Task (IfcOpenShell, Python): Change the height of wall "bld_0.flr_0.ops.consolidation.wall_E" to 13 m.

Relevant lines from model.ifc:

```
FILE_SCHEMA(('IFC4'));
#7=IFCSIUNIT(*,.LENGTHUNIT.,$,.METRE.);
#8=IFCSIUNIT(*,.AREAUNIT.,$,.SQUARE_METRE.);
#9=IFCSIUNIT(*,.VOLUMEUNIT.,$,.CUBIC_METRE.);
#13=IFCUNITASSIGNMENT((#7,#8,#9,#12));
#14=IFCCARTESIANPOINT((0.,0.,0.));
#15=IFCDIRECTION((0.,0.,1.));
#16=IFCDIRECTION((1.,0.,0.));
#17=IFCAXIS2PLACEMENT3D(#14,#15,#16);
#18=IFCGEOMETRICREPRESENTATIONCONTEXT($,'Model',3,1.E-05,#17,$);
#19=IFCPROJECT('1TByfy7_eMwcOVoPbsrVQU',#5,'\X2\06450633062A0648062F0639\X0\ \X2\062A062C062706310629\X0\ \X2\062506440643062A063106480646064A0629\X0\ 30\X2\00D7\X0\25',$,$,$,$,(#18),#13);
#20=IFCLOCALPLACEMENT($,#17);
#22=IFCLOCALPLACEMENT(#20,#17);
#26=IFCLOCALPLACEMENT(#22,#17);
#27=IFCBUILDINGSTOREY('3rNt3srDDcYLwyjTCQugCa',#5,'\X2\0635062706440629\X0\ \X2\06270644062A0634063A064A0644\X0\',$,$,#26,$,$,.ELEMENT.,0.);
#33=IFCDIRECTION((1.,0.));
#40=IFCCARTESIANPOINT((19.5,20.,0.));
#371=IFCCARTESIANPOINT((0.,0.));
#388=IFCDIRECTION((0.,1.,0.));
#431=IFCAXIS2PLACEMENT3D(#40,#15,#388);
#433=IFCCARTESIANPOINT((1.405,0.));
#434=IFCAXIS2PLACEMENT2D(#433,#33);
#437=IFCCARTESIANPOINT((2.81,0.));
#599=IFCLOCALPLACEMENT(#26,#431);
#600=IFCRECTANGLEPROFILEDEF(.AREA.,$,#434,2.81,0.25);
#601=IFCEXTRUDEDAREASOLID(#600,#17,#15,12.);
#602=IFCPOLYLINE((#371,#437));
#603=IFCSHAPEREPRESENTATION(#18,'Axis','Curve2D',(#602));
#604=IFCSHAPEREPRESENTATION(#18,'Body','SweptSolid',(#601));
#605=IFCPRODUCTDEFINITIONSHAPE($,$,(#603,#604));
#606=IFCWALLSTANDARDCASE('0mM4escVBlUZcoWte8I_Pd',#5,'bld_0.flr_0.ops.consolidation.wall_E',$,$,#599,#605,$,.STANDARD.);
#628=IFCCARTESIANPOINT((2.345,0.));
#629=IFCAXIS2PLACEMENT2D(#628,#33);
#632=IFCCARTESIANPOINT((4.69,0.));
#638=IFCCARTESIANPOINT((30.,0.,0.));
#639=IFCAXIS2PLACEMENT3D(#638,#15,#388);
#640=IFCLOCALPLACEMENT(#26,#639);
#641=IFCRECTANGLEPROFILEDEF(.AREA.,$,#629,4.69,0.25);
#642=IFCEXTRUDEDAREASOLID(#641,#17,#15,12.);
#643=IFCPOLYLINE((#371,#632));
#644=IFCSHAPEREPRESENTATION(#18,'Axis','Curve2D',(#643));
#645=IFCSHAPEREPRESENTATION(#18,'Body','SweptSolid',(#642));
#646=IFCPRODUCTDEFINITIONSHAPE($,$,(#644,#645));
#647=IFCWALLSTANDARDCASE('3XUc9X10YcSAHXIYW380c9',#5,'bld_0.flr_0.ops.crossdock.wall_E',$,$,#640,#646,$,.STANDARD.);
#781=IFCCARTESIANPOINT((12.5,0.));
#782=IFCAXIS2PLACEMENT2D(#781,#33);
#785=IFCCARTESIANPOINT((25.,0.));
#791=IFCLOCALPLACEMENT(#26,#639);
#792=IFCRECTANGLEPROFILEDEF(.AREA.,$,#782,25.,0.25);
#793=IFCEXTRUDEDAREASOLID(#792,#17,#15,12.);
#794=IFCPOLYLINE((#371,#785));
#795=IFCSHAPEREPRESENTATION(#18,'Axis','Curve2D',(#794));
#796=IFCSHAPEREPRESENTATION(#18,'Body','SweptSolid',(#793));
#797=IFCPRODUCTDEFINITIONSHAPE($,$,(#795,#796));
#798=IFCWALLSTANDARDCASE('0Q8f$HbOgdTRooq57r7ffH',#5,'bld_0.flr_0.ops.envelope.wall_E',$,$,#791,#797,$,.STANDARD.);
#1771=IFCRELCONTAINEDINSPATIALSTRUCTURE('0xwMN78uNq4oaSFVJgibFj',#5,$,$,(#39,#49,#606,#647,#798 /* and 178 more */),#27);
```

```python
import ifcopenshell
import ifcopenshell.geom
import ifcopenshell.util.shape

model = ifcopenshell.open("model.ifc")
settings = ifcopenshell.geom.settings()


def volume(element):
    """Net volume in cubic metres, openings subtracted."""
    shape = ifcopenshell.geom.create_shape(settings, element)
    return ifcopenshell.util.shape.get_volume(shape.geometry)


wall = model.by_guid("0mM4escVBlUZcoWte8I_Pd")
before = volume(wall)

body = next(r for r in wall.Representation.Representations if r.RepresentationIdentifier == "Body")
solid = body.Items[0]
old_height = solid.Depth
solid.Depth = 13.0
after = volume(wall)

print(f"height {old_height:g} -> {solid.Depth:g}, volume {before:.3f} -> {after:.3f} m3")

model.write("model_edited.ifc")
```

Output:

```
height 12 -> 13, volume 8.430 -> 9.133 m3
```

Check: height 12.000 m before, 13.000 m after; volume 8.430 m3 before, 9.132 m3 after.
